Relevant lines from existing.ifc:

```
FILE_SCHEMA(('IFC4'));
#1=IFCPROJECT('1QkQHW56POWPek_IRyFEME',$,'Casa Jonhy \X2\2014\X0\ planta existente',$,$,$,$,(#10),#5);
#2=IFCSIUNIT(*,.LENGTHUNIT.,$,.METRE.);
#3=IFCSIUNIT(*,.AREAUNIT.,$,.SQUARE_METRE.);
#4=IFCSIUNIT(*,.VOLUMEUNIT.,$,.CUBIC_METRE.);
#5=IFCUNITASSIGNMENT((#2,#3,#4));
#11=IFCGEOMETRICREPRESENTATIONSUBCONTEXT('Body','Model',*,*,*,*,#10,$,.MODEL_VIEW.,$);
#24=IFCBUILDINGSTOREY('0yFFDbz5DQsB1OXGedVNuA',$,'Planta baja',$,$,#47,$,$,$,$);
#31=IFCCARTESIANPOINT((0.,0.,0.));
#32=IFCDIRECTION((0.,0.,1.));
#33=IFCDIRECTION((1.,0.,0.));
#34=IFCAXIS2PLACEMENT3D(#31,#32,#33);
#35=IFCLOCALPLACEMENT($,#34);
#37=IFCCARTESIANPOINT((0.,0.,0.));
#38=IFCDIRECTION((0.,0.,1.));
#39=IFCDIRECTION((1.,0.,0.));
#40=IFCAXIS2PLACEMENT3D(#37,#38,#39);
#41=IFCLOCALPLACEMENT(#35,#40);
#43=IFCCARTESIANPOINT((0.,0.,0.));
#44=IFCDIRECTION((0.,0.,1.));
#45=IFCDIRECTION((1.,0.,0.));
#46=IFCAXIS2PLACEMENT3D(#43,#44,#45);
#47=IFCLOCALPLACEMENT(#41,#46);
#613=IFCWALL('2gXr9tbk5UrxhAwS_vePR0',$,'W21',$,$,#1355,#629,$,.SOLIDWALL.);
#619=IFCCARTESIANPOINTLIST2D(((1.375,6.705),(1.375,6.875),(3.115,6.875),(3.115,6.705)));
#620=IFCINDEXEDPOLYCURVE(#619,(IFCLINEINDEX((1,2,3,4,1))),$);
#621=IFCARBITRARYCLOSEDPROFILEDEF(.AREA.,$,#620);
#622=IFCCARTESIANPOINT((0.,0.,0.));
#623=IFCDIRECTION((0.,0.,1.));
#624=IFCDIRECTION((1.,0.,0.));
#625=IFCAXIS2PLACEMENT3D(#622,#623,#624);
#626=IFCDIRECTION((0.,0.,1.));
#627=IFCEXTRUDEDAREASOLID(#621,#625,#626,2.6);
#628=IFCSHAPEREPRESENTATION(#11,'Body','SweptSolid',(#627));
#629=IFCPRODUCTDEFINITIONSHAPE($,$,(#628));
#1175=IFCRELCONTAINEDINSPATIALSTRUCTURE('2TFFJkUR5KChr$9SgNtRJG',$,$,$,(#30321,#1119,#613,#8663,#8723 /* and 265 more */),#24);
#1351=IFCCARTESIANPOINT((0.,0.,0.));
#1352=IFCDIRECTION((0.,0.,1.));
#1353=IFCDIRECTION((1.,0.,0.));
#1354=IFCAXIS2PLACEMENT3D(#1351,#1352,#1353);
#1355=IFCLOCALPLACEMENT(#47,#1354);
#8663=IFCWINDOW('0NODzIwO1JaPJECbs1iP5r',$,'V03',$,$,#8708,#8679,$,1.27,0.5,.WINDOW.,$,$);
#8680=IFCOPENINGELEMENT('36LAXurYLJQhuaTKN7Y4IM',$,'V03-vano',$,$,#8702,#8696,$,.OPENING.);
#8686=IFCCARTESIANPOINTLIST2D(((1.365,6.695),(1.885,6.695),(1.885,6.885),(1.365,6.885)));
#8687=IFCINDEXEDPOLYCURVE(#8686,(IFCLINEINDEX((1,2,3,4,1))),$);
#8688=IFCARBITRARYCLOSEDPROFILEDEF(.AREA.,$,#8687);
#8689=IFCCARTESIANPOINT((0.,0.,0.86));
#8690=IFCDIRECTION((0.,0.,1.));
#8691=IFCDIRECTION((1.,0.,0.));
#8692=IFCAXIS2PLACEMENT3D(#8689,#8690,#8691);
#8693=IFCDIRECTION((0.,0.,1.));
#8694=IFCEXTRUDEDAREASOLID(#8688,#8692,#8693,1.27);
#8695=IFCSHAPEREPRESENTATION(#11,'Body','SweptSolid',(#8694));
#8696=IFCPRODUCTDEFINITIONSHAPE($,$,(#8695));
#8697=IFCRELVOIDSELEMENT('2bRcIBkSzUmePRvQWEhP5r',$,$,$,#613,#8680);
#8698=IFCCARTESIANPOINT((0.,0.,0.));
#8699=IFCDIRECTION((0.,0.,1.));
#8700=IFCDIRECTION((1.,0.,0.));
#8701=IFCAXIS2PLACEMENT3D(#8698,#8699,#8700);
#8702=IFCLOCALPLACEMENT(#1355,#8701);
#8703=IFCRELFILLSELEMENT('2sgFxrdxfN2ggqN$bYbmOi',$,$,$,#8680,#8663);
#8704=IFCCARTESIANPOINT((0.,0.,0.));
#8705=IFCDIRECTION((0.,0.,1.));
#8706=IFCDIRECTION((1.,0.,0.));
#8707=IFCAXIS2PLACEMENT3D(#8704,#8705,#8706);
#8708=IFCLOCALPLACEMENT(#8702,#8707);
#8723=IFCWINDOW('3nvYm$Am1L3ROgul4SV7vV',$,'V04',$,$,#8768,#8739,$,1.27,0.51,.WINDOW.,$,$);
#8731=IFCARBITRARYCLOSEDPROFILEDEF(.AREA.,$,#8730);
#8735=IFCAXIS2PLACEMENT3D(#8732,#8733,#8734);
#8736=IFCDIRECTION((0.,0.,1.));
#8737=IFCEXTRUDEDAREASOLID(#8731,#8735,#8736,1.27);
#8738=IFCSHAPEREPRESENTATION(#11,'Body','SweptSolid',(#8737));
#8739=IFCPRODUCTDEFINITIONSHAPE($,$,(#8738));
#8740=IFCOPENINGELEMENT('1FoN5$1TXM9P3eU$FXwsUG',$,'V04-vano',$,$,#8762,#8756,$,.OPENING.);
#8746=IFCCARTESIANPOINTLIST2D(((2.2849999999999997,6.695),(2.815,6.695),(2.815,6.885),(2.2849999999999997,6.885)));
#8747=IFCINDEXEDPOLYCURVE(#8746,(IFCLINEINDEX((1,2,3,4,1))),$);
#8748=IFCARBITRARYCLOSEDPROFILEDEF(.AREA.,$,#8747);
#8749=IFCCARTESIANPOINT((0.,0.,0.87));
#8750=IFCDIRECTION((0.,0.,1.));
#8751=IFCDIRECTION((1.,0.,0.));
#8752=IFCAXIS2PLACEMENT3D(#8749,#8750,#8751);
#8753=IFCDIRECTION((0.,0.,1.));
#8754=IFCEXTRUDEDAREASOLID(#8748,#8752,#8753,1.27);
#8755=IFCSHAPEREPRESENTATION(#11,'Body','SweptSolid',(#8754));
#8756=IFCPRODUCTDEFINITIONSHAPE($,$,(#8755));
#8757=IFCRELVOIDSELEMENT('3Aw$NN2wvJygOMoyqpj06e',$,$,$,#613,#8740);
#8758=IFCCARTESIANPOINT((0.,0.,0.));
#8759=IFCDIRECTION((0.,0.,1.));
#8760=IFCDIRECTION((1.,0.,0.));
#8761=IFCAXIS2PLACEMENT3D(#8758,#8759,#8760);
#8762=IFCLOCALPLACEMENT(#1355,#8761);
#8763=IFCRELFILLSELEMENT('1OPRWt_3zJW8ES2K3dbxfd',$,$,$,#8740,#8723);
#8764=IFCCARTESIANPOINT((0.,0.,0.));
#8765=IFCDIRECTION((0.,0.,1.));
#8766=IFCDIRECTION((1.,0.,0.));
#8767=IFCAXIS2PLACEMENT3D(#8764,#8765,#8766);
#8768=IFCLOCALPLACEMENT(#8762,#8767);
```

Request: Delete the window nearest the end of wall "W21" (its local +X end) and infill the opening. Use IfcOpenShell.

```python
import ifcopenshell
import ifcopenshell.api.feature
import ifcopenshell.api.root
import ifcopenshell.geom
import ifcopenshell.util.shape

model = ifcopenshell.open("existing.ifc")
settings = ifcopenshell.geom.settings()


def volume(element):
    """Net volume in cubic metres, openings subtracted."""
    shape = ifcopenshell.geom.create_shape(settings, element)
    return ifcopenshell.util.shape.get_volume(shape.geometry)


window = model.by_id(8723)
opening = window.FillsVoids[0].RelatingOpeningElement
wall = opening.VoidsElements[0].RelatingBuildingElement
before = volume(wall)

ifcopenshell.api.root.remove_product(model, product=window)
ifcopenshell.api.feature.remove_feature(model, feature=opening)

after = volume(wall)

print(f"wall volume {before:.3f} -> {after:.3f} m3")

model.write("existing_updated.ifc")
```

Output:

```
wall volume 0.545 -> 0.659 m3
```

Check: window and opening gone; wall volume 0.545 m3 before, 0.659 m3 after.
